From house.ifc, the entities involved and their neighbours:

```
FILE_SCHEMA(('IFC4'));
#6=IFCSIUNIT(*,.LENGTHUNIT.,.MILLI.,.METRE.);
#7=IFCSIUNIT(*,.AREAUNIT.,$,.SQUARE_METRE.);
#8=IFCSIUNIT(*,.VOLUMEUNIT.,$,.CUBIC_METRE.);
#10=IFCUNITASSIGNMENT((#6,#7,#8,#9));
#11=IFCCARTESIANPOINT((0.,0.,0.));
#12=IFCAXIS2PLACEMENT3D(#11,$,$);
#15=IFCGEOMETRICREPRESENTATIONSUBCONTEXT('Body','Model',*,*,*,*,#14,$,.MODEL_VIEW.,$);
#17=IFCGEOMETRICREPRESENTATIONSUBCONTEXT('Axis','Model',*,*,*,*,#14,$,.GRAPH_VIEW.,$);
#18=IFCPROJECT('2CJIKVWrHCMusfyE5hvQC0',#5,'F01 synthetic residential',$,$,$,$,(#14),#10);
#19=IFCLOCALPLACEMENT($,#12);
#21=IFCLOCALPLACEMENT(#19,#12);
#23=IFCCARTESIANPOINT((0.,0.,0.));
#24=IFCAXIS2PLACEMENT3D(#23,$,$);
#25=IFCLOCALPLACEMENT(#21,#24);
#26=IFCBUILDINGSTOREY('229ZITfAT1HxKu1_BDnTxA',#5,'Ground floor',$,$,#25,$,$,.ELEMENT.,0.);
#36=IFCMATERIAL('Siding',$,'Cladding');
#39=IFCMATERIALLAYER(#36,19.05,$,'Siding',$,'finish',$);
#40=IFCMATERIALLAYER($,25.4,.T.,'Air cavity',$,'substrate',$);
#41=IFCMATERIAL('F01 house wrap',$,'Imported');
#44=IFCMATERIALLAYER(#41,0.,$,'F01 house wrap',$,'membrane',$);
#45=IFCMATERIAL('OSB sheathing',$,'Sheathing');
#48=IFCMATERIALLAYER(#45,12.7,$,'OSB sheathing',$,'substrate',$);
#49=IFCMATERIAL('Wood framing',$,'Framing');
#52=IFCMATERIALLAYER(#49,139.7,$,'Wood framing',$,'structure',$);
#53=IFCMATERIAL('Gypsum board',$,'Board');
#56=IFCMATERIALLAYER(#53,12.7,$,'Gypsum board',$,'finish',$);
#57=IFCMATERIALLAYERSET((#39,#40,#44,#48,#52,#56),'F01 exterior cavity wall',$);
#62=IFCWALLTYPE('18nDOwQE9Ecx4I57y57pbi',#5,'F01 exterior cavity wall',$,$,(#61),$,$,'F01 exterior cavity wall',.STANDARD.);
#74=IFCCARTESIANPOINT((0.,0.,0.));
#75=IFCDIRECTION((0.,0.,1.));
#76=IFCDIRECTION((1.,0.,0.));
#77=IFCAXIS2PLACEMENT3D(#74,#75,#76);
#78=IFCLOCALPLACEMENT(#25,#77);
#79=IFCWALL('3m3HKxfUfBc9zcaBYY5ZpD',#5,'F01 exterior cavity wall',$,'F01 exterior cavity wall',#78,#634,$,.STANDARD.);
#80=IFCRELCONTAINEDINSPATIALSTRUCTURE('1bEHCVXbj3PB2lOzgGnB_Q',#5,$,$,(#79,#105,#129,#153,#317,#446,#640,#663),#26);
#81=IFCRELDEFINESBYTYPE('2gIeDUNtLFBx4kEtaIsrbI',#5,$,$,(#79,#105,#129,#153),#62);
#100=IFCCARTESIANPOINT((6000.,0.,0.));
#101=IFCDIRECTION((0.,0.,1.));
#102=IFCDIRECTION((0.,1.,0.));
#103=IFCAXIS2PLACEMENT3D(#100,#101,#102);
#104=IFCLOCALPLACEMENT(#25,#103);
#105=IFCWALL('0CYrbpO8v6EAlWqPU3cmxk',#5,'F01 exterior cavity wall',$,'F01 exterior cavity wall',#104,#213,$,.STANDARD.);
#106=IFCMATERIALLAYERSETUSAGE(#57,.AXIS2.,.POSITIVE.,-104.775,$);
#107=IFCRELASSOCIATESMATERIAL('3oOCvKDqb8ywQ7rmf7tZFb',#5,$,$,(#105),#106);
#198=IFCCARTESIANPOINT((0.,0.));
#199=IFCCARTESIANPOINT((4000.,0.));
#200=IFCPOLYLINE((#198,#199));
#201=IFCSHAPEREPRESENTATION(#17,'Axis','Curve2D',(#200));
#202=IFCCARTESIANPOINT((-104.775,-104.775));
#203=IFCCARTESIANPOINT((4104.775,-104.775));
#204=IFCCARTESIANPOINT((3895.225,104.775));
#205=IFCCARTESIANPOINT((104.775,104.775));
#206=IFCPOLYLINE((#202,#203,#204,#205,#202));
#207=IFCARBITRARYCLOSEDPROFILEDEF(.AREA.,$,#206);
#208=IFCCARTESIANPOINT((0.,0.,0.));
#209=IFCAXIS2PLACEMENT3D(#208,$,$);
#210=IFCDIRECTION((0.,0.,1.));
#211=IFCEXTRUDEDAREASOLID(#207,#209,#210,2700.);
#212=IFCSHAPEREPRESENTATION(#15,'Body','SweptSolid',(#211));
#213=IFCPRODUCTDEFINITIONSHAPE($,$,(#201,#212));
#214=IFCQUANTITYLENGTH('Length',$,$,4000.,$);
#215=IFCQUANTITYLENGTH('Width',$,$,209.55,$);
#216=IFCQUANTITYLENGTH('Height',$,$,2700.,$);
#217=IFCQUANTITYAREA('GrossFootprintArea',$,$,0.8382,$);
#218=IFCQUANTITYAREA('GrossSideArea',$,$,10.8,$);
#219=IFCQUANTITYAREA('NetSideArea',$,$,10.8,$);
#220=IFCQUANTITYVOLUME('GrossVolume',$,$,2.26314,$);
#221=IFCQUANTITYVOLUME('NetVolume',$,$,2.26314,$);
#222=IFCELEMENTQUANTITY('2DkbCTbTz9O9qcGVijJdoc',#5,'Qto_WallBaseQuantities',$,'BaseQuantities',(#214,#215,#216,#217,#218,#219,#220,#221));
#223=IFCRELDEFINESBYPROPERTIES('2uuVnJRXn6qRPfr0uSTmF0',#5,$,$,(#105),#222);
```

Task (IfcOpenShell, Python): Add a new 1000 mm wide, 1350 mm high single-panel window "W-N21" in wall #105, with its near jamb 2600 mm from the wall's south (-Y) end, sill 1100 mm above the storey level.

```python
import numpy as np
import ifcopenshell
import ifcopenshell.api.feature
import ifcopenshell.api.geometry
import ifcopenshell.api.pset
import ifcopenshell.api.root
import ifcopenshell.api.spatial
import ifcopenshell.geom
import ifcopenshell.util.element
import ifcopenshell.util.placement
import ifcopenshell.util.representation
import ifcopenshell.util.shape
import ifcopenshell.util.unit

model = ifcopenshell.open("house.ifc")
unit_scale = ifcopenshell.util.unit.calculate_unit_scale(model)
area_scale = ifcopenshell.util.unit.calculate_unit_scale(model, "AREAUNIT")
volume_scale = ifcopenshell.util.unit.calculate_unit_scale(model, "VOLUMEUNIT")
settings = ifcopenshell.geom.settings()


def volume(element):
    """Net volume in cubic metres, openings subtracted."""
    shape = ifcopenshell.geom.create_shape(settings, element)
    return ifcopenshell.util.shape.get_volume(shape.geometry)


wall = model.by_guid("0CYrbpO8v6EAlWqPU3cmxk")
storey = ifcopenshell.util.element.get_container(wall, ifc_class="IfcBuildingStorey")
context = ifcopenshell.util.representation.get_context(model, "Model", "Body", "MODEL_VIEW")
before = volume(wall)

width, height, from_end, sill = 1, 1.35, 2.6, 1.1  # metres

# The wall runs along its own X axis, and the end named is its -X end.
wall_shape = ifcopenshell.geom.create_shape(settings, wall)
x, y, z = ifcopenshell.util.shape.get_vertices(wall_shape.geometry).T
start = x.min() + from_end
face, thickness = float(y.min()), float(y.max() - y.min())
wall_matrix = ifcopenshell.util.placement.get_local_placement(wall.ObjectPlacement)
level = ifcopenshell.util.placement.get_local_placement(storey.ObjectPlacement)[2, 3]


def in_wall(x, y):
    """Placement at x, y metres in the wall's axes, at sill height."""
    matrix = wall_matrix.copy()
    matrix[:, 3] = wall_matrix @ np.array([x / unit_scale, y / unit_scale, 0.0, 1.0])
    matrix[2, 3] = level + sill / unit_scale
    return matrix


# Opening: a box that overshoots both wall faces by 50 mm.
opening = ifcopenshell.api.root.create_entity(model, ifc_class="IfcOpeningElement", predefined_type="OPENING")
box = ifcopenshell.api.geometry.add_wall_representation(
    model, context=context, length=width, height=height, thickness=thickness + 0.1
)
ifcopenshell.api.geometry.assign_representation(model, product=opening, representation=box)
ifcopenshell.api.geometry.edit_object_placement(model, product=opening, matrix=in_wall(start, face - 0.05), is_si=False)
ifcopenshell.api.feature.add_feature(model, feature=opening, element=wall)

window = ifcopenshell.api.root.create_entity(model, ifc_class="IfcWindow", name="W-N21", predefined_type="WINDOW")
window.OverallWidth, window.OverallHeight = width / unit_scale, height / unit_scale
window.PartitioningType = "SINGLE_PANEL"
body = ifcopenshell.api.geometry.add_window_representation(
    model,
    context=context,
    overall_width=window.OverallWidth,
    overall_height=window.OverallHeight,
    partition_type="SINGLE_PANEL",
)
ifcopenshell.api.geometry.assign_representation(model, product=window, representation=body)
ifcopenshell.api.spatial.assign_container(model, products=[window], relating_structure=storey)
ifcopenshell.api.feature.add_filling(model, opening=opening, element=window)

# Centre the window in the wall's thickness.
ifcopenshell.api.geometry.edit_object_placement(model, product=window, matrix=in_wall(start, face), is_si=False)
window_shape = ifcopenshell.geom.create_shape(settings, window)
depth = ifcopenshell.util.shape.get_vertices(window_shape.geometry)[:, 1]
offset = face + thickness / 2 - (depth.min() + depth.max()) / 2
ifcopenshell.api.geometry.edit_object_placement(model, product=window, matrix=in_wall(start, offset), is_si=False)

after = volume(wall)

# Update the wall's stored quantities.
qto = model.by_id(ifcopenshell.util.element.get_pset(wall, "Qto_WallBaseQuantities", should_inherit=False)["id"])
ifcopenshell.api.pset.edit_qto(model, qto=qto, properties={
    "NetSideArea": after / thickness / area_scale,
    "NetVolume": after / volume_scale,
})

print(f"wall volume {before:.3f} -> {after:.3f} m3")

model.write("house_updated.ifc")
```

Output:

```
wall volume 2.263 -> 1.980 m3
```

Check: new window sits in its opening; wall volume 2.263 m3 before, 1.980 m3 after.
